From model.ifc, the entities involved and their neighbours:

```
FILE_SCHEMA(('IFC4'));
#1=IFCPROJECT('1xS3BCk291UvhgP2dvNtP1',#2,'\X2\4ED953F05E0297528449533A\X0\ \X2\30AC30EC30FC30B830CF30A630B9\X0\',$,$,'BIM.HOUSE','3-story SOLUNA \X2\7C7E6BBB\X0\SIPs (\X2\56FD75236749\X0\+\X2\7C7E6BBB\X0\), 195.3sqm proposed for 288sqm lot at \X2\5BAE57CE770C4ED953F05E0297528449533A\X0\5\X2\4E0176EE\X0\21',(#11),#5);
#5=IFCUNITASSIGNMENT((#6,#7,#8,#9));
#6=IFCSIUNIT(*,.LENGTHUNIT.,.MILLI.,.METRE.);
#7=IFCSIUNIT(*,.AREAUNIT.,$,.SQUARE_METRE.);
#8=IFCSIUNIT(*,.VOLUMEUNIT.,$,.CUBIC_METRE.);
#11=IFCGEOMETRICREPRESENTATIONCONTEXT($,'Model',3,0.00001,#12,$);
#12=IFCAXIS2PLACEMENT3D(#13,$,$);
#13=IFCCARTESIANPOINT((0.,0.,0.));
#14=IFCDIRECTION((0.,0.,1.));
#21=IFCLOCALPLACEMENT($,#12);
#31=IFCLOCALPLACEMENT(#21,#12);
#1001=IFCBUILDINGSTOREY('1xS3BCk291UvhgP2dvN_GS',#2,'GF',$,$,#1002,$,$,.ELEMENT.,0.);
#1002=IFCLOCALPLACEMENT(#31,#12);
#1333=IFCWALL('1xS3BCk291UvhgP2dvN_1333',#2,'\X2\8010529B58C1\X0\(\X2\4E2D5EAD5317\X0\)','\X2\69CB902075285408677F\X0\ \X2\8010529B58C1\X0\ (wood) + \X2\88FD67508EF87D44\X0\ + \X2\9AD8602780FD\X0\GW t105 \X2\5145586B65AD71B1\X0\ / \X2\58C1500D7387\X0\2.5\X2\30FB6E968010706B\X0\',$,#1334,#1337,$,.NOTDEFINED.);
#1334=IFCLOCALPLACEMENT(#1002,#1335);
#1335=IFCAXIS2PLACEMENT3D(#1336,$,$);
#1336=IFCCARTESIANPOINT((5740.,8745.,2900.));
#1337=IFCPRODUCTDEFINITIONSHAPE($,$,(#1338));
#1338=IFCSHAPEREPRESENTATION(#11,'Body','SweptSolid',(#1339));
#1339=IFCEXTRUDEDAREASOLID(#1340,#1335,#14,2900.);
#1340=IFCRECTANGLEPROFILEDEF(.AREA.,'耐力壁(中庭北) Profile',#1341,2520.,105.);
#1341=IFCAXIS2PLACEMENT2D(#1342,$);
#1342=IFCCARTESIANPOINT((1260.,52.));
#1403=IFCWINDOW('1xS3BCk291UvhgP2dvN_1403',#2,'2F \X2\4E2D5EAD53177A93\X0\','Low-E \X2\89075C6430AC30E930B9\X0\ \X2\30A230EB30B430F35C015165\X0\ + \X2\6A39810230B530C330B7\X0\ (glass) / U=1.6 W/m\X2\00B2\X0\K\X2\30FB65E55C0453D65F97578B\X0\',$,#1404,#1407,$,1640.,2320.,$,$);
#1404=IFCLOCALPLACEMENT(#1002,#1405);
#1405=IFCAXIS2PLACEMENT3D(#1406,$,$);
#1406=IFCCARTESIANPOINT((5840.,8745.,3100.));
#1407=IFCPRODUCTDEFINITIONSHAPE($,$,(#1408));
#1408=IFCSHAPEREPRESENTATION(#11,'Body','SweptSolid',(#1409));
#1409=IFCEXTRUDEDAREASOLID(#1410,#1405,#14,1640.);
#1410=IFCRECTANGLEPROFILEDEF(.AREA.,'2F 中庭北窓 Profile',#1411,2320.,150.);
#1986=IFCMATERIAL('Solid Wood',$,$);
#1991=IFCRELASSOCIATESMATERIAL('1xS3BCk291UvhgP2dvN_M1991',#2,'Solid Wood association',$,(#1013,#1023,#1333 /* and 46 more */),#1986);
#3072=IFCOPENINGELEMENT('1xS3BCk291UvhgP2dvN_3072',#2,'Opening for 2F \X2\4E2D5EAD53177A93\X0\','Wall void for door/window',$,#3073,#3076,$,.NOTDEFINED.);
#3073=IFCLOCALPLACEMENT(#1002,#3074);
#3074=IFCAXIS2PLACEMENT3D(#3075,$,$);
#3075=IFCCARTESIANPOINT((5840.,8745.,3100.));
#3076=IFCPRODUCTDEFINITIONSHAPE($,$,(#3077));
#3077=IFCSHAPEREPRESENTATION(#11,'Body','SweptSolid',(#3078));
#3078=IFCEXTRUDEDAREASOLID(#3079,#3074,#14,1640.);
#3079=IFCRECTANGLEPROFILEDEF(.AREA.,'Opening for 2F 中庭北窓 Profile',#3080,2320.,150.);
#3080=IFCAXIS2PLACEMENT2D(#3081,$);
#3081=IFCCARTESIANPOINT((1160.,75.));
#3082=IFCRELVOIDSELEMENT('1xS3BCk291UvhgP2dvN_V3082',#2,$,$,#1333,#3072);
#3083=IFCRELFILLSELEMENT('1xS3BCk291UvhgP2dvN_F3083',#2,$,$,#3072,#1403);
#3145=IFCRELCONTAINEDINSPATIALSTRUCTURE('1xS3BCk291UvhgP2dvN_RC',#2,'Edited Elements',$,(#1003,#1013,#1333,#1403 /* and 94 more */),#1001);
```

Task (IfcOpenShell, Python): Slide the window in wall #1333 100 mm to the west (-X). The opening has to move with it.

```python
import ifcopenshell
import ifcopenshell.api.geometry
import ifcopenshell.util.placement

model = ifcopenshell.open("model.ifc")

window = model.by_guid("1xS3BCk291UvhgP2dvN_1403")
opening = window.FillsVoids[0].RelatingOpeningElement
wall = opening.VoidsElements[0].RelatingBuildingElement

wall_matrix = ifcopenshell.util.placement.get_local_placement(wall.ObjectPlacement)
shift = wall_matrix[:3, 0] * -100.0
before = ifcopenshell.util.placement.get_local_placement(window.ObjectPlacement)[:3, 3].copy()

# The window is not placed relative to its opening, so move both.
for product in (opening, window):
    matrix = ifcopenshell.util.placement.get_local_placement(product.ObjectPlacement)
    matrix[:3, 3] += shift
    ifcopenshell.api.geometry.edit_object_placement(model, product=product, matrix=matrix, is_si=False)

after = ifcopenshell.util.placement.get_local_placement(window.ObjectPlacement)[:3, 3]
print("window moved by", (after - before).round(3) + 0.0)

model.write("model_v2.ifc")
```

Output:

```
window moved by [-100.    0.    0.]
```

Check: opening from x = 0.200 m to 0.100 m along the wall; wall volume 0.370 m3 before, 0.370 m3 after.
